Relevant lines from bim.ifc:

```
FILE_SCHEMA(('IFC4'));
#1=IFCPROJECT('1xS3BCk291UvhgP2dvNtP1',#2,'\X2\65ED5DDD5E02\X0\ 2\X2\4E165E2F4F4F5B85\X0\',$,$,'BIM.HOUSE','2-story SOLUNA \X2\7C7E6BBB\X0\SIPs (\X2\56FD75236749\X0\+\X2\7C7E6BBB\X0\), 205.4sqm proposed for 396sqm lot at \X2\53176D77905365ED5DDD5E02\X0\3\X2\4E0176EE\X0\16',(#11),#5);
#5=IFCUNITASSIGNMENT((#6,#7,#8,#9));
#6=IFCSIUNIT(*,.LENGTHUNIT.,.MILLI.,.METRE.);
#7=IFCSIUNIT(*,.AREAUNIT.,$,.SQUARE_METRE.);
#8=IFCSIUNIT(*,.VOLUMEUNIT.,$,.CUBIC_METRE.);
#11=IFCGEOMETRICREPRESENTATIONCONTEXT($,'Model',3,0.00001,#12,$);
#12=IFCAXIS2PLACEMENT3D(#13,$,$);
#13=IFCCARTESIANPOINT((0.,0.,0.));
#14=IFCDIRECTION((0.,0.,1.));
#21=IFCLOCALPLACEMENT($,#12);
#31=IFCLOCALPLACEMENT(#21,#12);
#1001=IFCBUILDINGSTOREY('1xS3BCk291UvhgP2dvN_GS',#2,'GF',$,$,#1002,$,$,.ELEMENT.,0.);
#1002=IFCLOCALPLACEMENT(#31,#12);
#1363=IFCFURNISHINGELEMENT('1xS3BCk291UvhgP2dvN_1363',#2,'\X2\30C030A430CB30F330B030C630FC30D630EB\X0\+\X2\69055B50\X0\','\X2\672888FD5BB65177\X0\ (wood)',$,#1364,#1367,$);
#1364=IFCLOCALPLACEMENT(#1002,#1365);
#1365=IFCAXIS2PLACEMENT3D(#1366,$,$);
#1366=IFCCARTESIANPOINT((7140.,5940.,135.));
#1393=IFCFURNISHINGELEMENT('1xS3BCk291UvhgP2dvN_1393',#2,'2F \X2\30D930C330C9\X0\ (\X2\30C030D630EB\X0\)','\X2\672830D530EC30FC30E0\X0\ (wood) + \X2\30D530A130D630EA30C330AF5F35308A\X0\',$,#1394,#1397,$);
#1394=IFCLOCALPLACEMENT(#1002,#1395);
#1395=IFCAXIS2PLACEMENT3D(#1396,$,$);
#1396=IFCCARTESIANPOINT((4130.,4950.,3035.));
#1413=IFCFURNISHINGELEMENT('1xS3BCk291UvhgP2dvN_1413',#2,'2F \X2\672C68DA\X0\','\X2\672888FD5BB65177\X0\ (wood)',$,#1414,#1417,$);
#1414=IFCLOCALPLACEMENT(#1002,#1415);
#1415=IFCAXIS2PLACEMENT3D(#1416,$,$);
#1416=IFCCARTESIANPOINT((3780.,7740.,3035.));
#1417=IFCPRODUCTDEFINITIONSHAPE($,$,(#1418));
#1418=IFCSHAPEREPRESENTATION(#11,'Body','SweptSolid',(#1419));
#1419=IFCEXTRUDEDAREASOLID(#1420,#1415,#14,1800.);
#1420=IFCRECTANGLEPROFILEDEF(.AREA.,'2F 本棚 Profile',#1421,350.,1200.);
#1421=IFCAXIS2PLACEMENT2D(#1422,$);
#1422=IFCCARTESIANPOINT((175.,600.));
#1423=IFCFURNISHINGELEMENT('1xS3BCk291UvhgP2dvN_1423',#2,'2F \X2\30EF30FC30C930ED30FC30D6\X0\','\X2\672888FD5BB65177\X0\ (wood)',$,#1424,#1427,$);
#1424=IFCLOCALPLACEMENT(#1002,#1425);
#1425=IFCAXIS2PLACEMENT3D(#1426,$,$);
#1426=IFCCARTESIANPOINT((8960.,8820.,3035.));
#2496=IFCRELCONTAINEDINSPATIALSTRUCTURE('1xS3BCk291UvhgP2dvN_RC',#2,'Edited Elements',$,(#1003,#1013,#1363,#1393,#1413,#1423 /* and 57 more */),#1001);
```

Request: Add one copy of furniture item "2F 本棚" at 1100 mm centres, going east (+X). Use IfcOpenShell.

```python
import numpy as np
import ifcopenshell
import ifcopenshell.api.geometry
import ifcopenshell.api.root
import ifcopenshell.util.element
import ifcopenshell.util.placement
import ifcopenshell.util.unit

model = ifcopenshell.open("bim.ifc")
unit_scale = ifcopenshell.util.unit.calculate_unit_scale(model)


def reuse_history(source, copy):
    """copy_class also copies each property set's owner history, people and application; keep the originals."""
    for rel in copy.IsDefinedBy:
        if rel.is_a("IfcRelDefinesByProperties") and (history := rel.RelatingPropertyDefinition.OwnerHistory):
            rel.RelatingPropertyDefinition.OwnerHistory = source.OwnerHistory
            ifcopenshell.util.element.remove_deep2(model, history)


source = model.by_guid("1xS3BCk291UvhgP2dvN_1413")
base = ifcopenshell.util.placement.get_local_placement(source.ObjectPlacement)
step = np.array([1.0, 0.0, 0.0]) * 1.1 / unit_scale

for i in range(1, 2):
    copy = ifcopenshell.api.root.copy_class(model, product=source)
    copy.Representation = ifcopenshell.util.element.copy_deep(
        model, source.Representation, exclude=["IfcGeometricRepresentationContext", "IfcRepresentationMap"]
    )
    reuse_history(source, copy)
    matrix = base.copy()
    matrix[:3, 3] += i * step
    print("added at", matrix[:3, 3].round(3) + 0.0)
    ifcopenshell.api.geometry.edit_object_placement(model, product=copy, matrix=matrix, is_si=False)

model.write("bim_v2.ifc")
```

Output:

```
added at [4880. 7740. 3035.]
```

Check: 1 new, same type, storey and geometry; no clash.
